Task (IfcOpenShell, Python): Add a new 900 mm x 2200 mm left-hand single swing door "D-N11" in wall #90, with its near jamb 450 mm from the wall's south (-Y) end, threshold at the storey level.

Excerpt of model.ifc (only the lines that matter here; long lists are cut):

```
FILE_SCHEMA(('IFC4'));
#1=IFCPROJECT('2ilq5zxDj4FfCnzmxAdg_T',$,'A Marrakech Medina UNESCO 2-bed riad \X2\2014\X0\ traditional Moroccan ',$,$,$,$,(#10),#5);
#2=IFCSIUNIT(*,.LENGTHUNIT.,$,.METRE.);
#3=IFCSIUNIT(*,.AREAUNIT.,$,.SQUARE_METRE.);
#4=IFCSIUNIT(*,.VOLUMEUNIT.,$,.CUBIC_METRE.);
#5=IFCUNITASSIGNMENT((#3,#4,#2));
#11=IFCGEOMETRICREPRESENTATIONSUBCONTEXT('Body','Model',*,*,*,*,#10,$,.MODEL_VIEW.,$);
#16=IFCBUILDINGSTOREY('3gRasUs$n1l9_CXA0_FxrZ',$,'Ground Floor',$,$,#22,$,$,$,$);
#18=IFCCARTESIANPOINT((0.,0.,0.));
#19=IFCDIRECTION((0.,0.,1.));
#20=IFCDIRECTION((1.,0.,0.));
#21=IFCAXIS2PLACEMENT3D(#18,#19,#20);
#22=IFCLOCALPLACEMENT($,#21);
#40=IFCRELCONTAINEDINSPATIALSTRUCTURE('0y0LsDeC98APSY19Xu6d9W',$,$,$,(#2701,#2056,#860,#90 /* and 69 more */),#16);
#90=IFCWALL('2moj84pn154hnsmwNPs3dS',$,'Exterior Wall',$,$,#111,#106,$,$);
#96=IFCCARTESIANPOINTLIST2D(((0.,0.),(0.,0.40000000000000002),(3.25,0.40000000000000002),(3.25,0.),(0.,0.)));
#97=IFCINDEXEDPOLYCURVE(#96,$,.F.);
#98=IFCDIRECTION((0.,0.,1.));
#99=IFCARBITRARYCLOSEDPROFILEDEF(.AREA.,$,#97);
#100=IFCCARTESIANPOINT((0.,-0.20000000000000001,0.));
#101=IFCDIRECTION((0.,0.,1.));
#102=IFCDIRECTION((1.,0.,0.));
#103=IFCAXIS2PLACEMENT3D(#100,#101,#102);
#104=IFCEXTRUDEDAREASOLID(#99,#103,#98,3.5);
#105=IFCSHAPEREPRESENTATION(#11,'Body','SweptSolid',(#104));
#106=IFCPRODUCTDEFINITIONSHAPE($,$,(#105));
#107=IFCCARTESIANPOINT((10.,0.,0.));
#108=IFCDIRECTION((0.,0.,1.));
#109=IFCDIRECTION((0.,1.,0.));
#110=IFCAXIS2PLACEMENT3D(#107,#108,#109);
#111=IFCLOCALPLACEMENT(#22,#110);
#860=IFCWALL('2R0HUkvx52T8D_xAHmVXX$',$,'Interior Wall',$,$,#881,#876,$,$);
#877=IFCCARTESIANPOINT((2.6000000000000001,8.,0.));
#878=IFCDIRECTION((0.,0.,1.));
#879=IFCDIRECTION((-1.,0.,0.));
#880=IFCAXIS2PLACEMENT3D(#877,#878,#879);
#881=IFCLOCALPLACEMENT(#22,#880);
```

```python
import numpy as np
import ifcopenshell
import ifcopenshell.api.feature
import ifcopenshell.api.geometry
import ifcopenshell.api.root
import ifcopenshell.api.spatial
import ifcopenshell.geom
import ifcopenshell.util.element
import ifcopenshell.util.placement
import ifcopenshell.util.representation
import ifcopenshell.util.shape
import ifcopenshell.util.unit

model = ifcopenshell.open("model.ifc")
unit_scale = ifcopenshell.util.unit.calculate_unit_scale(model)
settings = ifcopenshell.geom.settings()


def volume(element):
    """Net volume in cubic metres, openings subtracted."""
    shape = ifcopenshell.geom.create_shape(settings, element)
    return ifcopenshell.util.shape.get_volume(shape.geometry)


wall = model.by_id(90)
storey = ifcopenshell.util.element.get_container(wall, ifc_class="IfcBuildingStorey")
context = ifcopenshell.util.representation.get_context(model, "Model", "Body", "MODEL_VIEW")
before = volume(wall)

width, height, from_end, sill = 0.9, 2.2, 0.45, 0.0  # metres

# The wall runs along its own X axis, and the end named is its -X end.
wall_shape = ifcopenshell.geom.create_shape(settings, wall)
x, y, z = ifcopenshell.util.shape.get_vertices(wall_shape.geometry).T
start = x.min() + from_end
face, thickness = float(y.min()), float(y.max() - y.min())
wall_matrix = ifcopenshell.util.placement.get_local_placement(wall.ObjectPlacement)
level = ifcopenshell.util.placement.get_local_placement(storey.ObjectPlacement)[2, 3]


def in_wall(x, y):
    """Placement at x, y metres in the wall's axes, at sill height."""
    matrix = wall_matrix.copy()
    matrix[:, 3] = wall_matrix @ np.array([x / unit_scale, y / unit_scale, 0.0, 1.0])
    matrix[2, 3] = level + sill / unit_scale
    return matrix


# Opening: a box that overshoots both wall faces by 50 mm.
opening = ifcopenshell.api.root.create_entity(model, ifc_class="IfcOpeningElement", predefined_type="OPENING")
box = ifcopenshell.api.geometry.add_wall_representation(
    model, context=context, length=width, height=height, thickness=thickness + 0.1
)
ifcopenshell.api.geometry.assign_representation(model, product=opening, representation=box)
ifcopenshell.api.geometry.edit_object_placement(model, product=opening, matrix=in_wall(start, face - 0.05), is_si=False)
ifcopenshell.api.feature.add_feature(model, feature=opening, element=wall)

door = ifcopenshell.api.root.create_entity(model, ifc_class="IfcDoor", name="D-N11", predefined_type="DOOR")
door.OverallWidth, door.OverallHeight = width / unit_scale, height / unit_scale
door.OperationType = "SINGLE_SWING_LEFT"
body = ifcopenshell.api.geometry.add_door_representation(
    model,
    context=context,
    overall_width=door.OverallWidth,
    overall_height=door.OverallHeight,
    operation_type="SINGLE_SWING_LEFT",
    lining_properties={"LiningDepth": thickness / unit_scale, "ThresholdDepth": thickness / unit_scale},
)
ifcopenshell.api.geometry.assign_representation(model, product=door, representation=body)
ifcopenshell.api.spatial.assign_container(model, products=[door], relating_structure=storey)
ifcopenshell.api.feature.add_filling(model, opening=opening, element=door)

# The lining spans the wall, so the door starts at the wall face.
ifcopenshell.api.geometry.edit_object_placement(model, product=door, matrix=in_wall(start, face), is_si=False)

after = volume(wall)

print(f"wall volume {before:.3f} -> {after:.3f} m3")

model.write("model_updated.ifc")
```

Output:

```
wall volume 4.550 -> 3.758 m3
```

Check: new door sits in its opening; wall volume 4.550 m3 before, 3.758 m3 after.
